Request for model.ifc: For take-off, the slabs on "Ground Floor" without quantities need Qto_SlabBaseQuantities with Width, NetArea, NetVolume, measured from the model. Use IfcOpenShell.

First a look at what the model holds.

```python
import ifcopenshell
import ifcopenshell.util.element
import ifcopenshell.util.unit

model = ifcopenshell.open("model.ifc")
print(model.schema)
for unit_type in ("LENGTHUNIT", "AREAUNIT", "VOLUMEUNIT"):
    print(unit_type, ifcopenshell.util.unit.calculate_unit_scale(model, unit_type))
storey = next(s for s in model.by_type("IfcBuildingStorey") if s.Name == "Ground Floor")
slabs = [e for e in ifcopenshell.util.element.get_decomposition(storey) if e.is_a("IfcSlab")]
for e in sorted(slabs, key=lambda e: e.id()):
    print(e.id(), e.is_a(), e.Name, list(ifcopenshell.util.element.get_psets(e, qtos_only=True)), sep=" | ")
```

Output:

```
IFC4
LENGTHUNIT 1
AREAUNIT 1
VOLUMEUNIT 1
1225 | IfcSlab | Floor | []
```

```python
import ifcopenshell
import ifcopenshell.api.pset
import ifcopenshell.geom
import ifcopenshell.util.element
import ifcopenshell.util.shape
import ifcopenshell.util.unit

model = ifcopenshell.open("model.ifc")
unit_scale = ifcopenshell.util.unit.calculate_unit_scale(model)
area_scale = ifcopenshell.util.unit.calculate_unit_scale(model, "AREAUNIT")
volume_scale = ifcopenshell.util.unit.calculate_unit_scale(model, "VOLUMEUNIT")
settings = ifcopenshell.geom.settings()

storey = next(s for s in model.by_type("IfcBuildingStorey") if s.Name == "Ground Floor")
slabs = [e for e in ifcopenshell.util.element.get_decomposition(storey) if e.is_a("IfcSlab")]

for e in sorted(slabs, key=lambda e: e.id()):
    if ifcopenshell.util.element.get_psets(e, qtos_only=True, should_inherit=False):
        continue
    # Geometry comes back in metres, in the element's own axes.
    shape = ifcopenshell.geom.create_shape(settings, e)
    values = {
        "Width": ifcopenshell.util.shape.get_z(shape.geometry) / unit_scale,
        "NetArea": ifcopenshell.util.shape.get_footprint_area(shape.geometry) / area_scale,
        "NetVolume": ifcopenshell.util.shape.get_volume(shape.geometry) / volume_scale,
    }
    qto = ifcopenshell.api.pset.add_qto(model, product=e, name="Qto_SlabBaseQuantities")
    ifcopenshell.api.pset.edit_qto(model, qto=qto, properties=values)
    print(e.id(), {k: round(v, 3) for k, v in values.items()})

model.write("model_updated.ifc")
```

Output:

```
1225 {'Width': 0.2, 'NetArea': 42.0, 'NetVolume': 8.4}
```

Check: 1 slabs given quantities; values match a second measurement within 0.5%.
